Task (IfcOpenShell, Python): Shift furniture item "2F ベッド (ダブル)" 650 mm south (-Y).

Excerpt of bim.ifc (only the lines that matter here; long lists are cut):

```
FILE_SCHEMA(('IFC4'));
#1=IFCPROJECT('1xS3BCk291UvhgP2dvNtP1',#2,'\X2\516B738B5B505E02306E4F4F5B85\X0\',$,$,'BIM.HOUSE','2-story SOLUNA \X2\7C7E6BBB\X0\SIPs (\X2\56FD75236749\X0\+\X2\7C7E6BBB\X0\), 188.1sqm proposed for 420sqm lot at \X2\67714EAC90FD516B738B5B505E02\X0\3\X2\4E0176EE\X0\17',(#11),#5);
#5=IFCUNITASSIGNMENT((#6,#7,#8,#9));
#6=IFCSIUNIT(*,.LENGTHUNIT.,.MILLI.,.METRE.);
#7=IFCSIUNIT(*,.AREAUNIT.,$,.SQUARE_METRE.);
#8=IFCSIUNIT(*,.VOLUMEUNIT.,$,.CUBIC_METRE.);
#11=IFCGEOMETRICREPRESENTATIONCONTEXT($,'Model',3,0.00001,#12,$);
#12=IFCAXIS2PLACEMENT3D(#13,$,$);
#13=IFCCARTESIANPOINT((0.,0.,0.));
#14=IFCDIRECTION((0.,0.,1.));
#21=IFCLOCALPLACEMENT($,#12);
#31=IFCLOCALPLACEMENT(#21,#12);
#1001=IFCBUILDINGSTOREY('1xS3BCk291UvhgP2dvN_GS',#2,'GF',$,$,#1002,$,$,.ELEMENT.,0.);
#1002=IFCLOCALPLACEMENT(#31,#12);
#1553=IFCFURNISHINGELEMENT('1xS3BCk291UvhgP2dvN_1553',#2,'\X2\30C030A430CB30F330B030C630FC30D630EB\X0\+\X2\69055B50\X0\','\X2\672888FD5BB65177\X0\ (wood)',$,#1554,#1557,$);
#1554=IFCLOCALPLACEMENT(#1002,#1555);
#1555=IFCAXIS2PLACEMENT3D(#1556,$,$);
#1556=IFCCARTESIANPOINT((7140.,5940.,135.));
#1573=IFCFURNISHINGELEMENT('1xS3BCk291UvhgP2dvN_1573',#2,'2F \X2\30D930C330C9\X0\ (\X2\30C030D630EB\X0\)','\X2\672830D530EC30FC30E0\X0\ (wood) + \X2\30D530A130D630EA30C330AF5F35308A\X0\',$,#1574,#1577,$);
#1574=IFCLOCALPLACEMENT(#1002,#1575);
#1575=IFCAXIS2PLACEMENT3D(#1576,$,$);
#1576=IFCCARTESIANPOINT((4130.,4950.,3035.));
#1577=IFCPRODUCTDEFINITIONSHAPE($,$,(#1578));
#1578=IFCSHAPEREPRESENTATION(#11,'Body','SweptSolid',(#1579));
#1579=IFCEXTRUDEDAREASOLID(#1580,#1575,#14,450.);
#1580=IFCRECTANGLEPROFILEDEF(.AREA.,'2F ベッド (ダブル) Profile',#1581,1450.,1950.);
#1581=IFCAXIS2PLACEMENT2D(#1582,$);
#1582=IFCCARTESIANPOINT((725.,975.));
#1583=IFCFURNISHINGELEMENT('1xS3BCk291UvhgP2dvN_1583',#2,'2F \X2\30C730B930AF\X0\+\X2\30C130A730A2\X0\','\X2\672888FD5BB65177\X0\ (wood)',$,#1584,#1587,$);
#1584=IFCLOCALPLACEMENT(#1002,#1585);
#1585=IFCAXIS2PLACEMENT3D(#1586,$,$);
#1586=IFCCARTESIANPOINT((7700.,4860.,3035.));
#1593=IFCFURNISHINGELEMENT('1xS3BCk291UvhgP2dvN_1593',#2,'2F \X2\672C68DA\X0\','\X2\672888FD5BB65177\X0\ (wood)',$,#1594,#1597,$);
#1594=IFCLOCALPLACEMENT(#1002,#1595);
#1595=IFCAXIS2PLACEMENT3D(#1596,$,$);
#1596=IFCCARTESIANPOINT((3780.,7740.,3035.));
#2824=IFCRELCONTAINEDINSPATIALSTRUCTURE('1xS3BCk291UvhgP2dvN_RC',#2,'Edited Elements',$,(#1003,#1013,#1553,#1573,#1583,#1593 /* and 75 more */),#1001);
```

```python
import ifcopenshell
import ifcopenshell.api.geometry
import ifcopenshell.util.placement

model = ifcopenshell.open("bim.ifc")

item = model.by_guid("1xS3BCk291UvhgP2dvN_1573")
matrix = ifcopenshell.util.placement.get_local_placement(item.ObjectPlacement)
matrix[1, 3] -= 650.0
ifcopenshell.api.geometry.edit_object_placement(model, product=item, matrix=matrix, is_si=False)

print(ifcopenshell.util.placement.get_local_placement(item.ObjectPlacement).round(3) + 0.0)

model.write("bim_v2.ifc")
```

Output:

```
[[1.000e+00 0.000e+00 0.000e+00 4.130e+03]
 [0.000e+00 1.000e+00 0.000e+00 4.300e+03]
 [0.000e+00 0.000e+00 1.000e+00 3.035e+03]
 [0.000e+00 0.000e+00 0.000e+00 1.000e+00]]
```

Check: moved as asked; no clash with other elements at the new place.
